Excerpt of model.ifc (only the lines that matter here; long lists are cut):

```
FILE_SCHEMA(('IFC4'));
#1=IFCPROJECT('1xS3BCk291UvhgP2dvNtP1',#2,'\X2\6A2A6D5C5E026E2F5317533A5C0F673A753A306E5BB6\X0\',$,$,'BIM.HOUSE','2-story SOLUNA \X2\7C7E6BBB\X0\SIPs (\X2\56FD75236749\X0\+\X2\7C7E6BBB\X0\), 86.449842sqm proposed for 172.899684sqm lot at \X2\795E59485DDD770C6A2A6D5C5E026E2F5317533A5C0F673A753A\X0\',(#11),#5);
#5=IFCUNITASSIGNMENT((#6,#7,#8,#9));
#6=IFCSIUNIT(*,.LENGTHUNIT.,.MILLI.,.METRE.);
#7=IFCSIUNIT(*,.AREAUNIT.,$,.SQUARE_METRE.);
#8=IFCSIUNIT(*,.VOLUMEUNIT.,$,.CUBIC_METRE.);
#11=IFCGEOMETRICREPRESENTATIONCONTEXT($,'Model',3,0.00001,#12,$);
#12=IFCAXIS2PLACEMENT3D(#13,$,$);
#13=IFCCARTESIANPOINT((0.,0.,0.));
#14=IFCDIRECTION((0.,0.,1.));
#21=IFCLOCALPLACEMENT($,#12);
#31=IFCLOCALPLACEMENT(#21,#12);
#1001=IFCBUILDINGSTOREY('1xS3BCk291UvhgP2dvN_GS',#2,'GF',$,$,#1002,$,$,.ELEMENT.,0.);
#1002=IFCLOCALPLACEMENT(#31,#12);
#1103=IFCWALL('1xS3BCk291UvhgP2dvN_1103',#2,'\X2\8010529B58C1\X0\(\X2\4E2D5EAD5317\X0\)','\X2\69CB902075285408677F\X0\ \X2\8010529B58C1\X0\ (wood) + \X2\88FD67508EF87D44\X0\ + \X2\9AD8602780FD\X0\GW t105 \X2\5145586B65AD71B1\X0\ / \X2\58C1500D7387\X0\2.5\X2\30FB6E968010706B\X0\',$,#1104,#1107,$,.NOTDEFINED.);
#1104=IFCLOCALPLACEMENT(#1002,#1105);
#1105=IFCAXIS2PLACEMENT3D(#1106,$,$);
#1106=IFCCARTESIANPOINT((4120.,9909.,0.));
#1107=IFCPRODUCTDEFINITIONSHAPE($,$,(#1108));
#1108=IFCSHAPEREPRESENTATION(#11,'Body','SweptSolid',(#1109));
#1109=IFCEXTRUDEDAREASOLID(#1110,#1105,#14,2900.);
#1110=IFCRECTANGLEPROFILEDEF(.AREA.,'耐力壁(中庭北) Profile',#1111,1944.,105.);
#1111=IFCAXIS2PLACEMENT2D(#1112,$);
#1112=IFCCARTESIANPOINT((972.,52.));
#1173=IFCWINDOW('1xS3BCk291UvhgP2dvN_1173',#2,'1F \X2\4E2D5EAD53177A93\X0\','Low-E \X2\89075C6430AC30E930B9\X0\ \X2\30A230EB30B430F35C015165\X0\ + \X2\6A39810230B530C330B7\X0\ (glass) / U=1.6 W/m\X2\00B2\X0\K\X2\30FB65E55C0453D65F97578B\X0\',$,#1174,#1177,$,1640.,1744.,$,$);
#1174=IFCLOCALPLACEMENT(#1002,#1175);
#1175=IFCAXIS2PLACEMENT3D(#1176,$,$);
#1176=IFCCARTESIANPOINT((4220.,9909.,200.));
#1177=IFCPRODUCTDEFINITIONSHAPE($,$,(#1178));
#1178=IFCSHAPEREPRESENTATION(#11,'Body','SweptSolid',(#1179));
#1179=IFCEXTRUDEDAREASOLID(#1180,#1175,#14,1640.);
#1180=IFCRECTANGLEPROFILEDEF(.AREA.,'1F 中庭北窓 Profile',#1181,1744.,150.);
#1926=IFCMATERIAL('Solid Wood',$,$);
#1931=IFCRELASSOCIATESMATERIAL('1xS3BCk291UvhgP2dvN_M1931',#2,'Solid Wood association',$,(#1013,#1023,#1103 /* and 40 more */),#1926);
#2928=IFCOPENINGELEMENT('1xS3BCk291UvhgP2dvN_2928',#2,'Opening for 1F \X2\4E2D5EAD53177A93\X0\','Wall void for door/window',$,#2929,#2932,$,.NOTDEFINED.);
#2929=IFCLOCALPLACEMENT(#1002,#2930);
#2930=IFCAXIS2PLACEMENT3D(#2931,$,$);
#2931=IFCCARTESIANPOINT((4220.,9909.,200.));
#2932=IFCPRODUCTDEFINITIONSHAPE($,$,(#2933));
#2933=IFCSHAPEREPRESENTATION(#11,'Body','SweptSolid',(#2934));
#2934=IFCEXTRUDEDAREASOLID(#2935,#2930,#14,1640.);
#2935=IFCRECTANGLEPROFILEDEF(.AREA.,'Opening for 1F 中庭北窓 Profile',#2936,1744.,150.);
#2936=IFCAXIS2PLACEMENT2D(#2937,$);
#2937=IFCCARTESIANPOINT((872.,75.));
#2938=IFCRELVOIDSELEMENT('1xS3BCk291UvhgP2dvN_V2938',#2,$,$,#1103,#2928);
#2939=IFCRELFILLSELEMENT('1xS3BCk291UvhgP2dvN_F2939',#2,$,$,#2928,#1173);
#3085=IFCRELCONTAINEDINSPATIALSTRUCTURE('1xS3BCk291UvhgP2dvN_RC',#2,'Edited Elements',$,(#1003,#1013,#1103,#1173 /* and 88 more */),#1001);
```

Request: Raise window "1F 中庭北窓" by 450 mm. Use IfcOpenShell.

```python
import numpy as np
import ifcopenshell
import ifcopenshell.api.geometry
import ifcopenshell.util.placement
import ifcopenshell.util.unit

model = ifcopenshell.open("model.ifc")
unit_scale = ifcopenshell.util.unit.calculate_unit_scale(model)

window = model.by_guid("1xS3BCk291UvhgP2dvN_1173")
opening = window.FillsVoids[0].RelatingOpeningElement
dz = 450.0

shift = np.array([0.0, 0.0, dz])
# The window is not placed relative to its opening, so move both.
for product in (opening, window):
    matrix = ifcopenshell.util.placement.get_local_placement(product.ObjectPlacement)
    matrix[:3, 3] += shift
    ifcopenshell.api.geometry.edit_object_placement(model, product=product, matrix=matrix, is_si=False)

print(f"moved by {dz * unit_scale:+.3f} m")

model.write("model_updated.ifc")
```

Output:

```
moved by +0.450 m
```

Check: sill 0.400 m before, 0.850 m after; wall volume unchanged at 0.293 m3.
